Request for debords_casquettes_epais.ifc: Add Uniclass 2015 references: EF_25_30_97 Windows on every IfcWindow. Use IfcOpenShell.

First a look at what the model holds.

```python
import ifcopenshell

model = ifcopenshell.open("debords_casquettes_epais.ifc")
print(model.schema)
print("classifications:", [c.Name for c in model.by_type("IfcClassification")])
for ifc_class in ("IfcDoor", "IfcRoof", "IfcStair", "IfcWall", "IfcWindow"):
    print(ifc_class, len(model.by_type(ifc_class)))
```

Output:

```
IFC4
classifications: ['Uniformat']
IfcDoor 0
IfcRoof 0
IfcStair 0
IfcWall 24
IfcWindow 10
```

```python
import ifcopenshell
import ifcopenshell.api.classification

model = ifcopenshell.open("debords_casquettes_epais.ifc")

system = ifcopenshell.api.classification.add_classification(model, classification="Uniclass 2015")

codes = {
    "IfcWindow": ("EF_25_30_97", "Windows"),
}
for ifc_class, (code, name) in codes.items():
    products = model.by_type(ifc_class)
    ifcopenshell.api.classification.add_reference(
        model, products=products, classification=system, identification=code, name=name
    )
    print(code, len(products))

model.write("debords_casquettes_epais_rev.ifc")
```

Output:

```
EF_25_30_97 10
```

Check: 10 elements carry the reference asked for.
